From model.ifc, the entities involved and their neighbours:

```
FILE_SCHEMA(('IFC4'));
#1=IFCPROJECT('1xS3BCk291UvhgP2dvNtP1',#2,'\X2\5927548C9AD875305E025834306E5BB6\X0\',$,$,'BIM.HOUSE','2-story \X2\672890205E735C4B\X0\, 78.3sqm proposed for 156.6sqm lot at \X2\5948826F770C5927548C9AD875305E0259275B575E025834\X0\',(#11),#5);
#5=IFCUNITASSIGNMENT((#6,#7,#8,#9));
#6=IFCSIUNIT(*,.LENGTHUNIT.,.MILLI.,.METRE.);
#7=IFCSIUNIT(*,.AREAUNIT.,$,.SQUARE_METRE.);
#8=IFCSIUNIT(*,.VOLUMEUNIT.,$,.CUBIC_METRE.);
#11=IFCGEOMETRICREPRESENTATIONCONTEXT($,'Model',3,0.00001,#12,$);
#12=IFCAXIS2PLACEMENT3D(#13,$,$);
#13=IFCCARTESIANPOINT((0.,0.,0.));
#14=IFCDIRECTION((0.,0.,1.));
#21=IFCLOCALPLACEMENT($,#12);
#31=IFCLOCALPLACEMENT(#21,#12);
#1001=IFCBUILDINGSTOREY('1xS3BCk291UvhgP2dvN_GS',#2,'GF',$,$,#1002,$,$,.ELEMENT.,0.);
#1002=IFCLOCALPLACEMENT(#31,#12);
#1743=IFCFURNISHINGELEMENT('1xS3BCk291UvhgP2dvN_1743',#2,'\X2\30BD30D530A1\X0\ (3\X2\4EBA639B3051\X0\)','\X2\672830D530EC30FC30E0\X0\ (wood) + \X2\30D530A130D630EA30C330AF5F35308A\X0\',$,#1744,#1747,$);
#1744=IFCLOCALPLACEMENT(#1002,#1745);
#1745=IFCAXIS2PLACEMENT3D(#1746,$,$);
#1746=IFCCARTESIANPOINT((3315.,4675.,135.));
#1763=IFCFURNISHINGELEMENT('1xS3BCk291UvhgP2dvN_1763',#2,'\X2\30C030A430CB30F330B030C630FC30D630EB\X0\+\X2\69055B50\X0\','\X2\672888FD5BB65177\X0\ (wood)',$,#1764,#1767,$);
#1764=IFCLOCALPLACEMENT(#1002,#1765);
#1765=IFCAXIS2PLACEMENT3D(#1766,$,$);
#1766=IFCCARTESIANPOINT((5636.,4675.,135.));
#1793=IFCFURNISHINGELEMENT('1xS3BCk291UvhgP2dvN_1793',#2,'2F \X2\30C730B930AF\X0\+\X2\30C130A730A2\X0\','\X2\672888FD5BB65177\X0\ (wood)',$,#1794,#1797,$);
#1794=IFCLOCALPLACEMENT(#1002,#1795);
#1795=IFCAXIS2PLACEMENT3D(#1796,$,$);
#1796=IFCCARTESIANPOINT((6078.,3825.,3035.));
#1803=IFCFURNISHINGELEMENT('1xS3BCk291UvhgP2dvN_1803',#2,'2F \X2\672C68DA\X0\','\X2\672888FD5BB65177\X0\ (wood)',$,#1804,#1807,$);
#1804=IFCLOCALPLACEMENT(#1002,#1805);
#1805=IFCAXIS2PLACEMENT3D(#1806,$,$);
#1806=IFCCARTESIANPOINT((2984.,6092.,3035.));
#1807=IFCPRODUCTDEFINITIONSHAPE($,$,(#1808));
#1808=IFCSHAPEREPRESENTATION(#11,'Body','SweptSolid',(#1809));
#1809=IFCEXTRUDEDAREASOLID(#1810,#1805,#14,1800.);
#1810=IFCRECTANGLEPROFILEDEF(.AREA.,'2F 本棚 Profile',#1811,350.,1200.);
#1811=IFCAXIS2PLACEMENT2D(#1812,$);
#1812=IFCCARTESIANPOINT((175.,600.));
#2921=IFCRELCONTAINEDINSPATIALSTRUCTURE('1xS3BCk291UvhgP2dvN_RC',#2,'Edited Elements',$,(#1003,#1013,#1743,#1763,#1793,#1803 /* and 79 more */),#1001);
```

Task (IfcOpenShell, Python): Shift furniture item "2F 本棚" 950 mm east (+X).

```python
import ifcopenshell
import ifcopenshell.api.geometry
import ifcopenshell.util.placement
import ifcopenshell.util.unit

model = ifcopenshell.open("model.ifc")
unit_scale = ifcopenshell.util.unit.calculate_unit_scale(model)

item = model.by_id(1803)
matrix = ifcopenshell.util.placement.get_local_placement(item.ObjectPlacement)
matrix[0, 3] += 0.95 / unit_scale
ifcopenshell.api.geometry.edit_object_placement(model, product=item, matrix=matrix, is_si=False)

print(ifcopenshell.util.placement.get_local_placement(item.ObjectPlacement).round(3) + 0.0)

model.write("model_rev.ifc")
```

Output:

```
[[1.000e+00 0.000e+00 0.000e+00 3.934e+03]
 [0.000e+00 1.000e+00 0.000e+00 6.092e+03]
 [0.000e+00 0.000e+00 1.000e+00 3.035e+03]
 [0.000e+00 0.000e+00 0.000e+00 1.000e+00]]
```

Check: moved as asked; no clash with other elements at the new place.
